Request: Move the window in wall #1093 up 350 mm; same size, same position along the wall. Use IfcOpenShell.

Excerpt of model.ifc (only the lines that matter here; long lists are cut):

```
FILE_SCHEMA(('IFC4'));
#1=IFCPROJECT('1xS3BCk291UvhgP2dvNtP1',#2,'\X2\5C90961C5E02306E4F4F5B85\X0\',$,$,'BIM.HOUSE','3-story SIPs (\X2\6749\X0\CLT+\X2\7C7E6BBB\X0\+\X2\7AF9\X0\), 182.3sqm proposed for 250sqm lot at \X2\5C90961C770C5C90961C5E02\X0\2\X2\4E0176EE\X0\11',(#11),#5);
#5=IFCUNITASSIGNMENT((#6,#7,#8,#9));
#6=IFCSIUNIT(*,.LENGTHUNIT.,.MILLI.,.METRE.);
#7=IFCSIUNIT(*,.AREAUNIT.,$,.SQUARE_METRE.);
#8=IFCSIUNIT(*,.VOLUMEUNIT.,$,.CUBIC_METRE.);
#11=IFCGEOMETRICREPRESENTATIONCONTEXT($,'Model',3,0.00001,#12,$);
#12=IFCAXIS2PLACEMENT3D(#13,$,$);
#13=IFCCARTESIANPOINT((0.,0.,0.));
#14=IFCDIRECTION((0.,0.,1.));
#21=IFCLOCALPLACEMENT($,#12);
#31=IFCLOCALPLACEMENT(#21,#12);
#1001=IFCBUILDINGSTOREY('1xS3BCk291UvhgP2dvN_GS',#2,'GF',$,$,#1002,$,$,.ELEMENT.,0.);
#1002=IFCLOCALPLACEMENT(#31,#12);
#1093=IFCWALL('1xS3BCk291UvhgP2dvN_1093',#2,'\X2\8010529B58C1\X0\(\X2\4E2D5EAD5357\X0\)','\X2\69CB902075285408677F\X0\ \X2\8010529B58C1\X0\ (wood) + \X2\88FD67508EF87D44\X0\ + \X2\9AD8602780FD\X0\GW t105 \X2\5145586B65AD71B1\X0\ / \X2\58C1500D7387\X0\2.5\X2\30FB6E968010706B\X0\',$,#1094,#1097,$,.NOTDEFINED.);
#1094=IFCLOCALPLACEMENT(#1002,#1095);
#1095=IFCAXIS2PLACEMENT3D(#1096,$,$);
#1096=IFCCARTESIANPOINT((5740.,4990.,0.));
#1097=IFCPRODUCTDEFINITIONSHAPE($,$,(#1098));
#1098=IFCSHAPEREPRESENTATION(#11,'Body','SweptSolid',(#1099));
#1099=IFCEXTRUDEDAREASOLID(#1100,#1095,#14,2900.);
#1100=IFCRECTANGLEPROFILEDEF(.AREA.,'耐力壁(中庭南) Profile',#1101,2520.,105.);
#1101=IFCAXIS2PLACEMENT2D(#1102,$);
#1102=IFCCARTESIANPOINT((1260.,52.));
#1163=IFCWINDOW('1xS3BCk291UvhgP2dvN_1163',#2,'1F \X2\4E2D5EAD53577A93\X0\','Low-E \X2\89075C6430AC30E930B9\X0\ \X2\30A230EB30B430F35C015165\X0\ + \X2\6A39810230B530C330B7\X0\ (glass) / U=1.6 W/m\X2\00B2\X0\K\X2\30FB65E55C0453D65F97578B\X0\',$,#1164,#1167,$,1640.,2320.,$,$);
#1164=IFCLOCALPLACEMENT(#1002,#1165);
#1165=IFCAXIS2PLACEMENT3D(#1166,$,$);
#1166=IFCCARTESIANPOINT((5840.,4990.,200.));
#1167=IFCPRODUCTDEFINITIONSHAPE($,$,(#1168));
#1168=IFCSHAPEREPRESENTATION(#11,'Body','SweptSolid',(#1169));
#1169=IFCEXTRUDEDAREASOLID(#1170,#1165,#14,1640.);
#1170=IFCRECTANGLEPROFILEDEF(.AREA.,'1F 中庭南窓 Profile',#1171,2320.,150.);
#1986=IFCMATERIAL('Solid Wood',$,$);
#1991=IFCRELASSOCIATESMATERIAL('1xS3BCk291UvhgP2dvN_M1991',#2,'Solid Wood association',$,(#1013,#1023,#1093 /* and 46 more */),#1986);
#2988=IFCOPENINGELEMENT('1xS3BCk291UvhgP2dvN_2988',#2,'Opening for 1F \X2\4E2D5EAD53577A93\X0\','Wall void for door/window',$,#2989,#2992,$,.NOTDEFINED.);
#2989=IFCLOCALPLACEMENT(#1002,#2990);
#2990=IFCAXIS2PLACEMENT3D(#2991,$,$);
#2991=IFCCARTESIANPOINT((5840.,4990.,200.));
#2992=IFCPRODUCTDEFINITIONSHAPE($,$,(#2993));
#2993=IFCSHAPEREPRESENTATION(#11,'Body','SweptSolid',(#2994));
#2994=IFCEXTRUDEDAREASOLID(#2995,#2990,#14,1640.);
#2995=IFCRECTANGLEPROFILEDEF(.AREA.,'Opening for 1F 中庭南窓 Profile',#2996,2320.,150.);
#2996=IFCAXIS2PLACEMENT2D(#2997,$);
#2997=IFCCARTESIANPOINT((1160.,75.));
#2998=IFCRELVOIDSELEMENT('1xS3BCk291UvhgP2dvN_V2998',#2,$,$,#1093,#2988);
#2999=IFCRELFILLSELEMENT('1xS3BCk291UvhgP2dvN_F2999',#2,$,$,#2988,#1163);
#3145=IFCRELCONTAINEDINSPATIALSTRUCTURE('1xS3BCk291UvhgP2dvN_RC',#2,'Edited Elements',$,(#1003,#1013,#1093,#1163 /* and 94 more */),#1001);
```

```python
import numpy as np
import ifcopenshell
import ifcopenshell.api.geometry
import ifcopenshell.util.placement
import ifcopenshell.util.unit

model = ifcopenshell.open("model.ifc")
unit_scale = ifcopenshell.util.unit.calculate_unit_scale(model)

window = model.by_guid("1xS3BCk291UvhgP2dvN_1163")
opening = window.FillsVoids[0].RelatingOpeningElement
dz = 0.35 / unit_scale

shift = np.array([0.0, 0.0, dz])
# The window is not placed relative to its opening, so move both.
for product in (opening, window):
    matrix = ifcopenshell.util.placement.get_local_placement(product.ObjectPlacement)
    matrix[:3, 3] += shift
    ifcopenshell.api.geometry.edit_object_placement(model, product=product, matrix=matrix, is_si=False)

print(f"moved by {dz * unit_scale:+.3f} m")

model.write("model_updated.ifc")
```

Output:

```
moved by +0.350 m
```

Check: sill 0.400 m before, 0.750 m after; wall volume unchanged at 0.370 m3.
